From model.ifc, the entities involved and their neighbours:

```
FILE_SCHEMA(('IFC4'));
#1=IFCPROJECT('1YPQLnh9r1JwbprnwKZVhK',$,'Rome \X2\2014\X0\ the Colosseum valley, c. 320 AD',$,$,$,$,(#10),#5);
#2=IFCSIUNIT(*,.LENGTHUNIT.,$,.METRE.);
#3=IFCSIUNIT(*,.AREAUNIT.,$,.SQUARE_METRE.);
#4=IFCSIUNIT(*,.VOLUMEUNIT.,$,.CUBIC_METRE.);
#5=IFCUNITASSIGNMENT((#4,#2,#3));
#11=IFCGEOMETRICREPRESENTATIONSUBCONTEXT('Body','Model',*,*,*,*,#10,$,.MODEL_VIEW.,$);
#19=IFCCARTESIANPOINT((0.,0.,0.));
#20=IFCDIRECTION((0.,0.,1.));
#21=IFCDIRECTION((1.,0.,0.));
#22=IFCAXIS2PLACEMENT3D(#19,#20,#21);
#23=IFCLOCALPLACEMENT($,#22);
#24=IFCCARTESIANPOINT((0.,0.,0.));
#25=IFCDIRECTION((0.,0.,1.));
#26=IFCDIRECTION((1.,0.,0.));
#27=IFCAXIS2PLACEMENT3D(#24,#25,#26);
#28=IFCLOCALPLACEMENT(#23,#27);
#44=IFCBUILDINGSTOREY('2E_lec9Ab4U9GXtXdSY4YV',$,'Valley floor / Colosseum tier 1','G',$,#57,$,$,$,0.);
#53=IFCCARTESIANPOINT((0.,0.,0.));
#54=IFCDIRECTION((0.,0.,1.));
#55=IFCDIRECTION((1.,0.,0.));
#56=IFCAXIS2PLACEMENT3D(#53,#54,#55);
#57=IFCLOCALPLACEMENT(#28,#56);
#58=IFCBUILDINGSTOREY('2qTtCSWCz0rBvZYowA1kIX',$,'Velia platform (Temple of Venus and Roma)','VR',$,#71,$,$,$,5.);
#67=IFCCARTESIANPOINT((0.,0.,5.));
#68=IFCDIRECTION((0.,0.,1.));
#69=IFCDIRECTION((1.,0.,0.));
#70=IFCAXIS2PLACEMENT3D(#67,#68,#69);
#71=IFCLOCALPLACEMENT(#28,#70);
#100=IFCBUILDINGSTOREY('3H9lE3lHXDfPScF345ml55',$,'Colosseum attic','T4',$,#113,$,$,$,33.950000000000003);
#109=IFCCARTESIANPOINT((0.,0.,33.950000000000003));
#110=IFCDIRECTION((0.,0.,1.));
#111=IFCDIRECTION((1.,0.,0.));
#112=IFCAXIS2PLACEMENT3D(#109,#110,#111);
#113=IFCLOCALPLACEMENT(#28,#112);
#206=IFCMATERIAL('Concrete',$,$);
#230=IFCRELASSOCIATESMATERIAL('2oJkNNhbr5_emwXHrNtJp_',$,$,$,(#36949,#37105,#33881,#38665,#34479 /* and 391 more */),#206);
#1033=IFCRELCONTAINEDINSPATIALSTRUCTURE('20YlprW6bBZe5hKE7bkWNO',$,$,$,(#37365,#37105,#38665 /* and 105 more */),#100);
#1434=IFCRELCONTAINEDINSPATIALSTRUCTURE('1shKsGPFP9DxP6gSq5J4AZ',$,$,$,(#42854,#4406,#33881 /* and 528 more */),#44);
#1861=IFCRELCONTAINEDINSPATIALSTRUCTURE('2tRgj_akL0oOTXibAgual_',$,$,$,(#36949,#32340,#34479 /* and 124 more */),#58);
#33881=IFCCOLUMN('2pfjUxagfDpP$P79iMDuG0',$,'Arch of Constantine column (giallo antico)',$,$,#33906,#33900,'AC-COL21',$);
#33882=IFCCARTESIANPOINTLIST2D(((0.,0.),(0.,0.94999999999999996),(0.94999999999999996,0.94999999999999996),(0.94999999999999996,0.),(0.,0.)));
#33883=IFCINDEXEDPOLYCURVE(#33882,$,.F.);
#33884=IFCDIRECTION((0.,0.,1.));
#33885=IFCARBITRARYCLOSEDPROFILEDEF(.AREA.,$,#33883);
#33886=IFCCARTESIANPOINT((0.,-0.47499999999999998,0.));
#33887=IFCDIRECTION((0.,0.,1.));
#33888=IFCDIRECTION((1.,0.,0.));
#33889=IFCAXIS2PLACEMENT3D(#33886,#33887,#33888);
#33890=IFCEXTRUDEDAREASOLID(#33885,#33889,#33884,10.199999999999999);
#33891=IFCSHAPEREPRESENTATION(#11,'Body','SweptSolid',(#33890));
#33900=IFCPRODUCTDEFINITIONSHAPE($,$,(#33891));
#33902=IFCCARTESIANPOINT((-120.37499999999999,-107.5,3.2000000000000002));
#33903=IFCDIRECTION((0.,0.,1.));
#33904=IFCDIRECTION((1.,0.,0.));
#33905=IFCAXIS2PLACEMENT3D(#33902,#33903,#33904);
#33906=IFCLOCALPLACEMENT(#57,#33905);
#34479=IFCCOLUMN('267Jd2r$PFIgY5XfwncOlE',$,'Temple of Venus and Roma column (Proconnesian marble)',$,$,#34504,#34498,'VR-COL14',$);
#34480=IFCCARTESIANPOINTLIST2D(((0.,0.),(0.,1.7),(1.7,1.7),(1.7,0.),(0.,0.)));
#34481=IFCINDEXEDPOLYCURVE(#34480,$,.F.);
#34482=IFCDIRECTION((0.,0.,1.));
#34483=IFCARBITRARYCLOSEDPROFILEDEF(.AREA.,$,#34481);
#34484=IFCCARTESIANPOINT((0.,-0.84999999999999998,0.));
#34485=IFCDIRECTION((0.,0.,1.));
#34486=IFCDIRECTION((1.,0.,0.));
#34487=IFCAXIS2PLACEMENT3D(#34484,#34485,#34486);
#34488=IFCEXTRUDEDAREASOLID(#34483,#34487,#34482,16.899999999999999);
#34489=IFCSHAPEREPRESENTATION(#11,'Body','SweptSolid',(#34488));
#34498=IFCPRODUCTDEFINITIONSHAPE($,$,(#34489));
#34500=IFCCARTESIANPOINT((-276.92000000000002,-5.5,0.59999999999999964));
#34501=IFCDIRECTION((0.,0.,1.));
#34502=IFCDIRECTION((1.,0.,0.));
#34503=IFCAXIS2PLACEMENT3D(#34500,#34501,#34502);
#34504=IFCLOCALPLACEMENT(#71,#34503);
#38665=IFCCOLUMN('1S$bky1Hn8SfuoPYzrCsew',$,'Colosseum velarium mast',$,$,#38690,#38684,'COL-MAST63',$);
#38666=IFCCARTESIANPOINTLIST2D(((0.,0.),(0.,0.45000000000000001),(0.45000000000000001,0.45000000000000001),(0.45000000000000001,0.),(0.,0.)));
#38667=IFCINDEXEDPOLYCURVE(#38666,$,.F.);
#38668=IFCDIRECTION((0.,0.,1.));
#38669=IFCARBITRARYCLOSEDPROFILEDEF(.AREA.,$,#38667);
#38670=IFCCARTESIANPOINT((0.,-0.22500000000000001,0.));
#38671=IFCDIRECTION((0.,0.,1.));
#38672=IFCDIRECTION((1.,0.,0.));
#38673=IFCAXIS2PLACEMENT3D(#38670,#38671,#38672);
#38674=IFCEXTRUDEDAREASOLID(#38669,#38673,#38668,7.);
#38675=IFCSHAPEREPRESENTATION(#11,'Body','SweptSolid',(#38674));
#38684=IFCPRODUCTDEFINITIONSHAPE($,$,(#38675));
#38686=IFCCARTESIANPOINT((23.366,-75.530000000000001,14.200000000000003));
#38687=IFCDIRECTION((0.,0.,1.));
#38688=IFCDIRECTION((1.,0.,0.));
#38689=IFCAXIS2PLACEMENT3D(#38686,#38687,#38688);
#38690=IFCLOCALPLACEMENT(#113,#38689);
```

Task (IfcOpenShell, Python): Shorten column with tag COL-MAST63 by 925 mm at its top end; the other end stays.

```python
import ifcopenshell
import ifcopenshell.util.representation
import ifcopenshell.util.unit

model = ifcopenshell.open("model.ifc")
unit_scale = ifcopenshell.util.unit.calculate_unit_scale(model)

member = model.by_guid("1S$bky1Hn8SfuoPYzrCsew")
change = -0.925 / unit_scale

# The extrusion runs towards the end named, so only its depth changes.
body = ifcopenshell.util.representation.get_representation(member, "Model", "Body")
solid = body.Items[0]
old_length = solid.Depth
solid.Depth += change

print(f"length {old_length:g} -> {solid.Depth:g}")

model.write("model_rev.ifc")
```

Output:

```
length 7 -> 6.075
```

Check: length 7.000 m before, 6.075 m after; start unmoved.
